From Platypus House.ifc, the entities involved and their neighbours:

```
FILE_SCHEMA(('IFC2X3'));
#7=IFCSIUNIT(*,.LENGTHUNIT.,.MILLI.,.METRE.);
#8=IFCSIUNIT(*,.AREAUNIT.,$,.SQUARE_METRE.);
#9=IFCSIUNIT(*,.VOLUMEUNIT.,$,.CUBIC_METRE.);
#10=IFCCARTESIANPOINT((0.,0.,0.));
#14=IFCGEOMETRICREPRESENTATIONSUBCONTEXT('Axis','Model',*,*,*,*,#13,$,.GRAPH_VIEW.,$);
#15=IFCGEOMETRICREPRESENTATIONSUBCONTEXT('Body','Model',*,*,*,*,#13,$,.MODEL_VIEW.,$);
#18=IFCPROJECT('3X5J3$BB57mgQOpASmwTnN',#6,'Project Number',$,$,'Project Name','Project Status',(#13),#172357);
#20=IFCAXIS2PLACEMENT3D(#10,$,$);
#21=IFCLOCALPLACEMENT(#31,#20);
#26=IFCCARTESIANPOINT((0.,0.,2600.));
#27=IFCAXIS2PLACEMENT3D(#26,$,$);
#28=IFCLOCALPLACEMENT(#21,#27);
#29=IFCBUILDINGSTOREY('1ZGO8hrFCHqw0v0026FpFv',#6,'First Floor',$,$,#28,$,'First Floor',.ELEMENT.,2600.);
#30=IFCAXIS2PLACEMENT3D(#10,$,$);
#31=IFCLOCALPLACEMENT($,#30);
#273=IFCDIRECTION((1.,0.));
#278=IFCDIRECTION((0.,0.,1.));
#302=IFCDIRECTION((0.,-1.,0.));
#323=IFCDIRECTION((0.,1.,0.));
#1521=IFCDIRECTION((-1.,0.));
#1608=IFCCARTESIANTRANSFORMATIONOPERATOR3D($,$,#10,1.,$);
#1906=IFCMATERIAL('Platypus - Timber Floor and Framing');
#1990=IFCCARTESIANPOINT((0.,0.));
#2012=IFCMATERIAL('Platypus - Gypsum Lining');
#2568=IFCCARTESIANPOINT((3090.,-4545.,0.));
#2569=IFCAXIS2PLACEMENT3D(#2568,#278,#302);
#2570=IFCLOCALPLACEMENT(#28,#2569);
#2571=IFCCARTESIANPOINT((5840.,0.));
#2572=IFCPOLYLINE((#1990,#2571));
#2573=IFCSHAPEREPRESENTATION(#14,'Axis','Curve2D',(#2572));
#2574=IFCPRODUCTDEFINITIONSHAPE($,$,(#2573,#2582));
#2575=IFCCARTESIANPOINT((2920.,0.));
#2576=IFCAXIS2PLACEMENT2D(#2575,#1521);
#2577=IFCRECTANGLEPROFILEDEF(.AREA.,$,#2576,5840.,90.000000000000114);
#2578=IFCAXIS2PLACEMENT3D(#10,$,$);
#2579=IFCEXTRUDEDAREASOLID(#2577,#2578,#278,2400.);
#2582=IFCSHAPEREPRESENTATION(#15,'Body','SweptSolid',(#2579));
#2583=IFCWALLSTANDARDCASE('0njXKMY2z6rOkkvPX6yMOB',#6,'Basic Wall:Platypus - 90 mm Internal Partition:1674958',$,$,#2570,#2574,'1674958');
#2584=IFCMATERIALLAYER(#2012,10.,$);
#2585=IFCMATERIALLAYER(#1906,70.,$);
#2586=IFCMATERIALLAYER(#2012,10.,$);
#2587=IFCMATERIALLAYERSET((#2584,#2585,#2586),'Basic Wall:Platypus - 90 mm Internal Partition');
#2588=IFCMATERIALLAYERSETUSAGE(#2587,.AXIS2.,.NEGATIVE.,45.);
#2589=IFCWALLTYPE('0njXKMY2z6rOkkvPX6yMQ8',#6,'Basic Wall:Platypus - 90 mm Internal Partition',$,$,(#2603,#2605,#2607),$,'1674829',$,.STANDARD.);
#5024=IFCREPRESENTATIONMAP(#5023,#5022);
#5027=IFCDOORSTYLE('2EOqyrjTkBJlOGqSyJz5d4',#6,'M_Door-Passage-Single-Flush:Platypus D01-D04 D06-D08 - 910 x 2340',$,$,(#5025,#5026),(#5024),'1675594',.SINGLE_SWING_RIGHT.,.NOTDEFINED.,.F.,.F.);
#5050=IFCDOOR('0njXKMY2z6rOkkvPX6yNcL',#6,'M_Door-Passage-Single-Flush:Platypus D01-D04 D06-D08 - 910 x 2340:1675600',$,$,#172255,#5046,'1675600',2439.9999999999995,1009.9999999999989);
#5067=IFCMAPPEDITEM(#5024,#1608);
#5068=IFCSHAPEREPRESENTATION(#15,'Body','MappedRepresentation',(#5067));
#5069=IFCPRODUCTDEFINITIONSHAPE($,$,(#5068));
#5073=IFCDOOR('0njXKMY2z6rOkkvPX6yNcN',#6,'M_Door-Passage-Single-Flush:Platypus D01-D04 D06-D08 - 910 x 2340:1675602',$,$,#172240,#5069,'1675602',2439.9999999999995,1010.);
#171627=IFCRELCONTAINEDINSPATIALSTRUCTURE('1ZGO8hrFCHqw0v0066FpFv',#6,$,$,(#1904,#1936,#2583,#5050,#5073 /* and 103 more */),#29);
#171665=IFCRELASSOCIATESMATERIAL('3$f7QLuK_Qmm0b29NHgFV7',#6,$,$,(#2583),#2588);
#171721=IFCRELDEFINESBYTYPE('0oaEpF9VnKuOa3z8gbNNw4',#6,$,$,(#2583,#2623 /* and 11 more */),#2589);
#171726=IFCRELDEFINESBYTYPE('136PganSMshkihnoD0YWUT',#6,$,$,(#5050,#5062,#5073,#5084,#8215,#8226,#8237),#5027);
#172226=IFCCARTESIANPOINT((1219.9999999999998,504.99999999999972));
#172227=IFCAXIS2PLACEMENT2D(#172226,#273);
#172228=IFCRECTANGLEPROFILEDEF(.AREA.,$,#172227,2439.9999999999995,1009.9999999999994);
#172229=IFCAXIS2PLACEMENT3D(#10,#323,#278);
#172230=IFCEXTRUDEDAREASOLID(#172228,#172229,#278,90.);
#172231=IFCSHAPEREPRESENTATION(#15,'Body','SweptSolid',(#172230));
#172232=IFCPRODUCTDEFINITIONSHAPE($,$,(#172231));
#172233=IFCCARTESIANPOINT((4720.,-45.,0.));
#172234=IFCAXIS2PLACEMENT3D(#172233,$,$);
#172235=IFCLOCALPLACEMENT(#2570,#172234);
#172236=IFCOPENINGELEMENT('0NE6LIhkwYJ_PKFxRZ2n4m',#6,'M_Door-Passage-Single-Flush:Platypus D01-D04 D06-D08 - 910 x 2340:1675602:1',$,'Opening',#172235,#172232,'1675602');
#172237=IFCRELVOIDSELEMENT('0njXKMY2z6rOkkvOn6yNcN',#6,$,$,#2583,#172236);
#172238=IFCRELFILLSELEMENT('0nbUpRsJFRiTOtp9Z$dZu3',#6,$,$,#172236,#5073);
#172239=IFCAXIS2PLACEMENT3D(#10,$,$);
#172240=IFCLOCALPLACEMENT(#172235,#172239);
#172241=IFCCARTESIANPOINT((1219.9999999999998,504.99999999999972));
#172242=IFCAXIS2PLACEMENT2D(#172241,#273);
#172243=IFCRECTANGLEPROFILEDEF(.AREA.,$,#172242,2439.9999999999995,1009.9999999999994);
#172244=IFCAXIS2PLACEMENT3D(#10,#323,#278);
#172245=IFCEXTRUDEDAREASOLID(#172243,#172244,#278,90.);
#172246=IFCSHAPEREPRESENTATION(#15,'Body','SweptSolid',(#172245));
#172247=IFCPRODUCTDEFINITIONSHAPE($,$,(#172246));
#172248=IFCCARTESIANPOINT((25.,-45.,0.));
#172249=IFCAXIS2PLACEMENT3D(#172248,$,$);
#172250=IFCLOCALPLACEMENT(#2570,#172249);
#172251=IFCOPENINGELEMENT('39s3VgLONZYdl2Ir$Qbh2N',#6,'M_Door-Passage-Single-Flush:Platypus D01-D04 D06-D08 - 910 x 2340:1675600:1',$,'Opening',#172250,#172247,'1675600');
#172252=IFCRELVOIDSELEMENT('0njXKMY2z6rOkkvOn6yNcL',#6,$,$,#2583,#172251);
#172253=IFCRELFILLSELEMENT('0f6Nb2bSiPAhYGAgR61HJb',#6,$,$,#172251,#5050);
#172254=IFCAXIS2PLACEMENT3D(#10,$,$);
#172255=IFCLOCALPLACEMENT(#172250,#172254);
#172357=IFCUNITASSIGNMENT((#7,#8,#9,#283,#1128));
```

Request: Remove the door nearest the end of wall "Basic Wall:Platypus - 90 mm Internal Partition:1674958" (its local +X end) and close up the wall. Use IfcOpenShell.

```python
import ifcopenshell
import ifcopenshell.api.feature
import ifcopenshell.api.root
import ifcopenshell.geom
import ifcopenshell.util.shape

model = ifcopenshell.open("Platypus House.ifc")
settings = ifcopenshell.geom.settings()


def volume(element):
    """Net volume in cubic metres, openings subtracted."""
    shape = ifcopenshell.geom.create_shape(settings, element)
    return ifcopenshell.util.shape.get_volume(shape.geometry)


door = model.by_id(5073)
opening = door.FillsVoids[0].RelatingOpeningElement
wall = opening.VoidsElements[0].RelatingBuildingElement
before = volume(wall)

ifcopenshell.api.root.remove_product(model, product=door)
ifcopenshell.api.feature.remove_feature(model, feature=opening)

after = volume(wall)

print(f"wall volume {before:.3f} -> {after:.3f} m3")

model.write("Platypus House-out.ifc")
```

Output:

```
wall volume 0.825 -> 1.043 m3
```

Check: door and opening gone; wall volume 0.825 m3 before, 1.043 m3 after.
